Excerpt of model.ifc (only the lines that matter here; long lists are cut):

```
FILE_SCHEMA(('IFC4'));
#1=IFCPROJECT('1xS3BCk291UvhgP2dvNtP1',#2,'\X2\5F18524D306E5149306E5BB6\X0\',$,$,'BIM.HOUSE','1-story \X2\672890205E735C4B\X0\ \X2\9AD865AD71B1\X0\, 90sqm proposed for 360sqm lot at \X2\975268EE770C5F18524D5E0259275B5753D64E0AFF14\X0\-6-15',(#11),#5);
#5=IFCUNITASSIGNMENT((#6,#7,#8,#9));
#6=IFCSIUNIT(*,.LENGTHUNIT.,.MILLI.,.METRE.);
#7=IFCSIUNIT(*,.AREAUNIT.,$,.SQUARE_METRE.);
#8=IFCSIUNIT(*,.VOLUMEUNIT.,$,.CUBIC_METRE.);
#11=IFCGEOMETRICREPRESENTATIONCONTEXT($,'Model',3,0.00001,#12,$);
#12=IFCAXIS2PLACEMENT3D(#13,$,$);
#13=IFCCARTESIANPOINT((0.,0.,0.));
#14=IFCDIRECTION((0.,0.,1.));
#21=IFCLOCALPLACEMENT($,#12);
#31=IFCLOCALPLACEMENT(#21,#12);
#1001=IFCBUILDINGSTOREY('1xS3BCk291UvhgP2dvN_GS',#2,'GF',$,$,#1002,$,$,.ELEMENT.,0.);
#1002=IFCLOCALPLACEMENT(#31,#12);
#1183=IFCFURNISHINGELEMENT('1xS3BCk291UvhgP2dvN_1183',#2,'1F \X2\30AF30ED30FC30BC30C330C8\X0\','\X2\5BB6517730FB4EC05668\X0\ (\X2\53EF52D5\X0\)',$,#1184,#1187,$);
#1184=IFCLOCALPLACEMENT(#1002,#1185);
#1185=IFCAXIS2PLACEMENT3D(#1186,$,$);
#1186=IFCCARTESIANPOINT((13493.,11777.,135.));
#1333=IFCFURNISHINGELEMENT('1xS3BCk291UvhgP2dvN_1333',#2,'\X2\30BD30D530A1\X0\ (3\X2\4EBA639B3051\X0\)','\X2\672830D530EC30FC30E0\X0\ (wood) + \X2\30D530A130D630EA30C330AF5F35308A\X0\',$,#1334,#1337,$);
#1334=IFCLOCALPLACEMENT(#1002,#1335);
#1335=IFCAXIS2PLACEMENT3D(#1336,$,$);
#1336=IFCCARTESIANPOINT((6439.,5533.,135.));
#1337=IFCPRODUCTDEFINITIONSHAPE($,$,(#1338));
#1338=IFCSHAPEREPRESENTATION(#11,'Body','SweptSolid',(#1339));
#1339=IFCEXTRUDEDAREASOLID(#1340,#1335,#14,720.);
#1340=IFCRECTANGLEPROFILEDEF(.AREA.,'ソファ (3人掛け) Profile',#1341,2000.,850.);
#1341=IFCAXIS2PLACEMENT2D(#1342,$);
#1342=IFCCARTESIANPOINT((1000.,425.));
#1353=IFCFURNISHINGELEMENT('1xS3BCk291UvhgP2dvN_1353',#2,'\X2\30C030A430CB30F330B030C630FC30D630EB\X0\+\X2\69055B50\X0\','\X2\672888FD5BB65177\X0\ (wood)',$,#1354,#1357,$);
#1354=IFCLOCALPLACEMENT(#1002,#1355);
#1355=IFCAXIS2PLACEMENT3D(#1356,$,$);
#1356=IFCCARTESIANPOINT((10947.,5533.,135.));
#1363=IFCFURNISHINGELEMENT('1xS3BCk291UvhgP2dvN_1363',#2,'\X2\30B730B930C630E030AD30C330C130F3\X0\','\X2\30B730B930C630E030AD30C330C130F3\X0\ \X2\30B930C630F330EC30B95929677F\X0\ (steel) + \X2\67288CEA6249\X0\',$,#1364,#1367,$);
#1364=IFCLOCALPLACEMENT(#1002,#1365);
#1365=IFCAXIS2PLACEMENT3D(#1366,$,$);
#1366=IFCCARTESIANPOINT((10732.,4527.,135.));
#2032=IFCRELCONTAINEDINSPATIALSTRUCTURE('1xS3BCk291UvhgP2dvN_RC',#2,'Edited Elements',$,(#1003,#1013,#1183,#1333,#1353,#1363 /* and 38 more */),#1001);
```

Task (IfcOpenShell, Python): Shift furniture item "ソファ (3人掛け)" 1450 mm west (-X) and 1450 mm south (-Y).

```python
import ifcopenshell
import ifcopenshell.api.geometry
import ifcopenshell.util.placement

model = ifcopenshell.open("model.ifc")

item = model.by_guid("1xS3BCk291UvhgP2dvN_1333")
matrix = ifcopenshell.util.placement.get_local_placement(item.ObjectPlacement)
matrix[0, 3] -= 1450.0
matrix[1, 3] -= 1450.0
ifcopenshell.api.geometry.edit_object_placement(model, product=item, matrix=matrix, is_si=False)

print(ifcopenshell.util.placement.get_local_placement(item.ObjectPlacement).round(3) + 0.0)

model.write("model-out.ifc")
```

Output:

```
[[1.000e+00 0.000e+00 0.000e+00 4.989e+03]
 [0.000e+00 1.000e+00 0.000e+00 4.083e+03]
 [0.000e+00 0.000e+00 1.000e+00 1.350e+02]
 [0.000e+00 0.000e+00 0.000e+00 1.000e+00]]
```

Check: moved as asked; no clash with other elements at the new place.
